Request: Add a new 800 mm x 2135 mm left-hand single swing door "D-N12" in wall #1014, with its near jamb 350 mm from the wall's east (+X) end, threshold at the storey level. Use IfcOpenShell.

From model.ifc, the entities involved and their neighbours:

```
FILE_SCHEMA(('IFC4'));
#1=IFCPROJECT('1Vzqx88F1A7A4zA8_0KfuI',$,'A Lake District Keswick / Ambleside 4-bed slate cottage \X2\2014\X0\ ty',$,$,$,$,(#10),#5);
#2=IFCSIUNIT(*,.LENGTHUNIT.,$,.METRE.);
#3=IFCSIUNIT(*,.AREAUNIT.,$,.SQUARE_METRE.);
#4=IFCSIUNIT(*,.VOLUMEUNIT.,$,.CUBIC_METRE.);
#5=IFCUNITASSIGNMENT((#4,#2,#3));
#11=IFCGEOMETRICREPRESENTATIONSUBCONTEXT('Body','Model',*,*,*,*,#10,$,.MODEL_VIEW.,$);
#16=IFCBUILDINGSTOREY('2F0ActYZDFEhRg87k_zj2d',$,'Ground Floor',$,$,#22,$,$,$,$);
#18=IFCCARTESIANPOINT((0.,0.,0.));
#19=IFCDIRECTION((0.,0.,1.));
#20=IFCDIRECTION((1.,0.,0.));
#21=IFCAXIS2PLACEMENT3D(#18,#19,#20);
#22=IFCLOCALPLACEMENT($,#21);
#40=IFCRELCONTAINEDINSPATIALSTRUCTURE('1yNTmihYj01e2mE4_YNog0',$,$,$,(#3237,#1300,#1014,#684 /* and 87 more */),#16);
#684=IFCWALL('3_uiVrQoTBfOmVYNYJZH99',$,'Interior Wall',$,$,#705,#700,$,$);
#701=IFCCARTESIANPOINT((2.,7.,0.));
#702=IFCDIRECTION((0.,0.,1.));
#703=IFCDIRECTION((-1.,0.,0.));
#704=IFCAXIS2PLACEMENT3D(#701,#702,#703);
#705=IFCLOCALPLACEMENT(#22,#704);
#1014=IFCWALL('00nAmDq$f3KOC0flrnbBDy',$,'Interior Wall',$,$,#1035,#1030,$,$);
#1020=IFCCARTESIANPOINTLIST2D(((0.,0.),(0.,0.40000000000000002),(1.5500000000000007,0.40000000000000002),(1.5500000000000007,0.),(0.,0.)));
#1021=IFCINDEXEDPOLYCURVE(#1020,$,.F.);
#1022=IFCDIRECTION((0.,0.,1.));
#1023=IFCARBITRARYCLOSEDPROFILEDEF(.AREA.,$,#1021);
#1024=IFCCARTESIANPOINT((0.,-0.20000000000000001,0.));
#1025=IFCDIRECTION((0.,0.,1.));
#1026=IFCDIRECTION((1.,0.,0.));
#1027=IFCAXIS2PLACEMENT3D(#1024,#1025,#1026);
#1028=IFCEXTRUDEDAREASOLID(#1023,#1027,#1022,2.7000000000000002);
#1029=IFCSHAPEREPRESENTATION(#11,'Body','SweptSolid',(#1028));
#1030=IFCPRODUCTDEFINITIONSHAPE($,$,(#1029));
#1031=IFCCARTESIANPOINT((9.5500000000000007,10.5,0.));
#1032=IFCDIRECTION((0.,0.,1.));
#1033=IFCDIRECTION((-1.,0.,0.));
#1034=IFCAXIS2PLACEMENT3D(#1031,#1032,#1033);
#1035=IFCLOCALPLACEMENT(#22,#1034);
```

```python
import numpy as np
import ifcopenshell
import ifcopenshell.api.feature
import ifcopenshell.api.geometry
import ifcopenshell.api.root
import ifcopenshell.api.spatial
import ifcopenshell.geom
import ifcopenshell.util.element
import ifcopenshell.util.placement
import ifcopenshell.util.representation
import ifcopenshell.util.shape
import ifcopenshell.util.unit

model = ifcopenshell.open("model.ifc")
unit_scale = ifcopenshell.util.unit.calculate_unit_scale(model)
settings = ifcopenshell.geom.settings()


def volume(element):
    """Net volume in cubic metres, openings subtracted."""
    shape = ifcopenshell.geom.create_shape(settings, element)
    return ifcopenshell.util.shape.get_volume(shape.geometry)


wall = model.by_guid("00nAmDq$f3KOC0flrnbBDy")
storey = ifcopenshell.util.element.get_container(wall, ifc_class="IfcBuildingStorey")
context = ifcopenshell.util.representation.get_context(model, "Model", "Body", "MODEL_VIEW")
before = volume(wall)

width, height, from_end, sill = 0.8, 2.135, 0.35, 0.0  # metres

# The wall runs along its own X axis, and the end named is its -X end.
wall_shape = ifcopenshell.geom.create_shape(settings, wall)
x, y, z = ifcopenshell.util.shape.get_vertices(wall_shape.geometry).T
start = x.min() + from_end
face, thickness = float(y.min()), float(y.max() - y.min())
wall_matrix = ifcopenshell.util.placement.get_local_placement(wall.ObjectPlacement)
level = ifcopenshell.util.placement.get_local_placement(storey.ObjectPlacement)[2, 3]


def in_wall(x, y):
    """Placement at x, y metres in the wall's axes, at sill height."""
    matrix = wall_matrix.copy()
    matrix[:, 3] = wall_matrix @ np.array([x / unit_scale, y / unit_scale, 0.0, 1.0])
    matrix[2, 3] = level + sill / unit_scale
    return matrix


# Opening: a box that overshoots both wall faces by 50 mm.
opening = ifcopenshell.api.root.create_entity(model, ifc_class="IfcOpeningElement", predefined_type="OPENING")
box = ifcopenshell.api.geometry.add_wall_representation(
    model, context=context, length=width, height=height, thickness=thickness + 0.1
)
ifcopenshell.api.geometry.assign_representation(model, product=opening, representation=box)
ifcopenshell.api.geometry.edit_object_placement(model, product=opening, matrix=in_wall(start, face - 0.05), is_si=False)
ifcopenshell.api.feature.add_feature(model, feature=opening, element=wall)

door = ifcopenshell.api.root.create_entity(model, ifc_class="IfcDoor", name="D-N12", predefined_type="DOOR")
door.OverallWidth, door.OverallHeight = width / unit_scale, height / unit_scale
door.OperationType = "SINGLE_SWING_LEFT"
body = ifcopenshell.api.geometry.add_door_representation(
    model,
    context=context,
    overall_width=door.OverallWidth,
    overall_height=door.OverallHeight,
    operation_type="SINGLE_SWING_LEFT",
    lining_properties={"LiningDepth": thickness / unit_scale, "ThresholdDepth": thickness / unit_scale},
)
ifcopenshell.api.geometry.assign_representation(model, product=door, representation=body)
ifcopenshell.api.spatial.assign_container(model, products=[door], relating_structure=storey)
ifcopenshell.api.feature.add_filling(model, opening=opening, element=door)

# The lining spans the wall, so the door starts at the wall face.
ifcopenshell.api.geometry.edit_object_placement(model, product=door, matrix=in_wall(start, face), is_si=False)

after = volume(wall)

print(f"wall volume {before:.3f} -> {after:.3f} m3")

model.write("model_v2.ifc")
```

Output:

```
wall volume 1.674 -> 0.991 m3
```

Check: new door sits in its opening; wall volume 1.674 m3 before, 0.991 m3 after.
